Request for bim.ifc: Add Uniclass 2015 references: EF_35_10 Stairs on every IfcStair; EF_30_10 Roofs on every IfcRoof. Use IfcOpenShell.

First a look at what the model holds.

```python
import ifcopenshell

model = ifcopenshell.open("bim.ifc")
print(model.schema)
print("classifications:", [c.Name for c in model.by_type("IfcClassification")])
for ifc_class in ("IfcDoor", "IfcRoof", "IfcStair", "IfcWall", "IfcWindow"):
    print(ifc_class, len(model.by_type(ifc_class)))
```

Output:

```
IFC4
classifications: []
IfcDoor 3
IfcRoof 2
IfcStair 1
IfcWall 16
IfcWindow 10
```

```python
import ifcopenshell
import ifcopenshell.api.classification

model = ifcopenshell.open("bim.ifc")

system = ifcopenshell.api.classification.add_classification(model, classification="Uniclass 2015")

codes = {
    "IfcStair": ("EF_35_10", "Stairs"),
    "IfcRoof": ("EF_30_10", "Roofs"),
}
for ifc_class, (code, name) in codes.items():
    products = model.by_type(ifc_class)
    ifcopenshell.api.classification.add_reference(
        model, products=products, classification=system, identification=code, name=name
    )
    print(code, len(products))

model.write("bim_edited.ifc")
```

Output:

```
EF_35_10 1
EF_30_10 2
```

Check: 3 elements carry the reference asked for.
